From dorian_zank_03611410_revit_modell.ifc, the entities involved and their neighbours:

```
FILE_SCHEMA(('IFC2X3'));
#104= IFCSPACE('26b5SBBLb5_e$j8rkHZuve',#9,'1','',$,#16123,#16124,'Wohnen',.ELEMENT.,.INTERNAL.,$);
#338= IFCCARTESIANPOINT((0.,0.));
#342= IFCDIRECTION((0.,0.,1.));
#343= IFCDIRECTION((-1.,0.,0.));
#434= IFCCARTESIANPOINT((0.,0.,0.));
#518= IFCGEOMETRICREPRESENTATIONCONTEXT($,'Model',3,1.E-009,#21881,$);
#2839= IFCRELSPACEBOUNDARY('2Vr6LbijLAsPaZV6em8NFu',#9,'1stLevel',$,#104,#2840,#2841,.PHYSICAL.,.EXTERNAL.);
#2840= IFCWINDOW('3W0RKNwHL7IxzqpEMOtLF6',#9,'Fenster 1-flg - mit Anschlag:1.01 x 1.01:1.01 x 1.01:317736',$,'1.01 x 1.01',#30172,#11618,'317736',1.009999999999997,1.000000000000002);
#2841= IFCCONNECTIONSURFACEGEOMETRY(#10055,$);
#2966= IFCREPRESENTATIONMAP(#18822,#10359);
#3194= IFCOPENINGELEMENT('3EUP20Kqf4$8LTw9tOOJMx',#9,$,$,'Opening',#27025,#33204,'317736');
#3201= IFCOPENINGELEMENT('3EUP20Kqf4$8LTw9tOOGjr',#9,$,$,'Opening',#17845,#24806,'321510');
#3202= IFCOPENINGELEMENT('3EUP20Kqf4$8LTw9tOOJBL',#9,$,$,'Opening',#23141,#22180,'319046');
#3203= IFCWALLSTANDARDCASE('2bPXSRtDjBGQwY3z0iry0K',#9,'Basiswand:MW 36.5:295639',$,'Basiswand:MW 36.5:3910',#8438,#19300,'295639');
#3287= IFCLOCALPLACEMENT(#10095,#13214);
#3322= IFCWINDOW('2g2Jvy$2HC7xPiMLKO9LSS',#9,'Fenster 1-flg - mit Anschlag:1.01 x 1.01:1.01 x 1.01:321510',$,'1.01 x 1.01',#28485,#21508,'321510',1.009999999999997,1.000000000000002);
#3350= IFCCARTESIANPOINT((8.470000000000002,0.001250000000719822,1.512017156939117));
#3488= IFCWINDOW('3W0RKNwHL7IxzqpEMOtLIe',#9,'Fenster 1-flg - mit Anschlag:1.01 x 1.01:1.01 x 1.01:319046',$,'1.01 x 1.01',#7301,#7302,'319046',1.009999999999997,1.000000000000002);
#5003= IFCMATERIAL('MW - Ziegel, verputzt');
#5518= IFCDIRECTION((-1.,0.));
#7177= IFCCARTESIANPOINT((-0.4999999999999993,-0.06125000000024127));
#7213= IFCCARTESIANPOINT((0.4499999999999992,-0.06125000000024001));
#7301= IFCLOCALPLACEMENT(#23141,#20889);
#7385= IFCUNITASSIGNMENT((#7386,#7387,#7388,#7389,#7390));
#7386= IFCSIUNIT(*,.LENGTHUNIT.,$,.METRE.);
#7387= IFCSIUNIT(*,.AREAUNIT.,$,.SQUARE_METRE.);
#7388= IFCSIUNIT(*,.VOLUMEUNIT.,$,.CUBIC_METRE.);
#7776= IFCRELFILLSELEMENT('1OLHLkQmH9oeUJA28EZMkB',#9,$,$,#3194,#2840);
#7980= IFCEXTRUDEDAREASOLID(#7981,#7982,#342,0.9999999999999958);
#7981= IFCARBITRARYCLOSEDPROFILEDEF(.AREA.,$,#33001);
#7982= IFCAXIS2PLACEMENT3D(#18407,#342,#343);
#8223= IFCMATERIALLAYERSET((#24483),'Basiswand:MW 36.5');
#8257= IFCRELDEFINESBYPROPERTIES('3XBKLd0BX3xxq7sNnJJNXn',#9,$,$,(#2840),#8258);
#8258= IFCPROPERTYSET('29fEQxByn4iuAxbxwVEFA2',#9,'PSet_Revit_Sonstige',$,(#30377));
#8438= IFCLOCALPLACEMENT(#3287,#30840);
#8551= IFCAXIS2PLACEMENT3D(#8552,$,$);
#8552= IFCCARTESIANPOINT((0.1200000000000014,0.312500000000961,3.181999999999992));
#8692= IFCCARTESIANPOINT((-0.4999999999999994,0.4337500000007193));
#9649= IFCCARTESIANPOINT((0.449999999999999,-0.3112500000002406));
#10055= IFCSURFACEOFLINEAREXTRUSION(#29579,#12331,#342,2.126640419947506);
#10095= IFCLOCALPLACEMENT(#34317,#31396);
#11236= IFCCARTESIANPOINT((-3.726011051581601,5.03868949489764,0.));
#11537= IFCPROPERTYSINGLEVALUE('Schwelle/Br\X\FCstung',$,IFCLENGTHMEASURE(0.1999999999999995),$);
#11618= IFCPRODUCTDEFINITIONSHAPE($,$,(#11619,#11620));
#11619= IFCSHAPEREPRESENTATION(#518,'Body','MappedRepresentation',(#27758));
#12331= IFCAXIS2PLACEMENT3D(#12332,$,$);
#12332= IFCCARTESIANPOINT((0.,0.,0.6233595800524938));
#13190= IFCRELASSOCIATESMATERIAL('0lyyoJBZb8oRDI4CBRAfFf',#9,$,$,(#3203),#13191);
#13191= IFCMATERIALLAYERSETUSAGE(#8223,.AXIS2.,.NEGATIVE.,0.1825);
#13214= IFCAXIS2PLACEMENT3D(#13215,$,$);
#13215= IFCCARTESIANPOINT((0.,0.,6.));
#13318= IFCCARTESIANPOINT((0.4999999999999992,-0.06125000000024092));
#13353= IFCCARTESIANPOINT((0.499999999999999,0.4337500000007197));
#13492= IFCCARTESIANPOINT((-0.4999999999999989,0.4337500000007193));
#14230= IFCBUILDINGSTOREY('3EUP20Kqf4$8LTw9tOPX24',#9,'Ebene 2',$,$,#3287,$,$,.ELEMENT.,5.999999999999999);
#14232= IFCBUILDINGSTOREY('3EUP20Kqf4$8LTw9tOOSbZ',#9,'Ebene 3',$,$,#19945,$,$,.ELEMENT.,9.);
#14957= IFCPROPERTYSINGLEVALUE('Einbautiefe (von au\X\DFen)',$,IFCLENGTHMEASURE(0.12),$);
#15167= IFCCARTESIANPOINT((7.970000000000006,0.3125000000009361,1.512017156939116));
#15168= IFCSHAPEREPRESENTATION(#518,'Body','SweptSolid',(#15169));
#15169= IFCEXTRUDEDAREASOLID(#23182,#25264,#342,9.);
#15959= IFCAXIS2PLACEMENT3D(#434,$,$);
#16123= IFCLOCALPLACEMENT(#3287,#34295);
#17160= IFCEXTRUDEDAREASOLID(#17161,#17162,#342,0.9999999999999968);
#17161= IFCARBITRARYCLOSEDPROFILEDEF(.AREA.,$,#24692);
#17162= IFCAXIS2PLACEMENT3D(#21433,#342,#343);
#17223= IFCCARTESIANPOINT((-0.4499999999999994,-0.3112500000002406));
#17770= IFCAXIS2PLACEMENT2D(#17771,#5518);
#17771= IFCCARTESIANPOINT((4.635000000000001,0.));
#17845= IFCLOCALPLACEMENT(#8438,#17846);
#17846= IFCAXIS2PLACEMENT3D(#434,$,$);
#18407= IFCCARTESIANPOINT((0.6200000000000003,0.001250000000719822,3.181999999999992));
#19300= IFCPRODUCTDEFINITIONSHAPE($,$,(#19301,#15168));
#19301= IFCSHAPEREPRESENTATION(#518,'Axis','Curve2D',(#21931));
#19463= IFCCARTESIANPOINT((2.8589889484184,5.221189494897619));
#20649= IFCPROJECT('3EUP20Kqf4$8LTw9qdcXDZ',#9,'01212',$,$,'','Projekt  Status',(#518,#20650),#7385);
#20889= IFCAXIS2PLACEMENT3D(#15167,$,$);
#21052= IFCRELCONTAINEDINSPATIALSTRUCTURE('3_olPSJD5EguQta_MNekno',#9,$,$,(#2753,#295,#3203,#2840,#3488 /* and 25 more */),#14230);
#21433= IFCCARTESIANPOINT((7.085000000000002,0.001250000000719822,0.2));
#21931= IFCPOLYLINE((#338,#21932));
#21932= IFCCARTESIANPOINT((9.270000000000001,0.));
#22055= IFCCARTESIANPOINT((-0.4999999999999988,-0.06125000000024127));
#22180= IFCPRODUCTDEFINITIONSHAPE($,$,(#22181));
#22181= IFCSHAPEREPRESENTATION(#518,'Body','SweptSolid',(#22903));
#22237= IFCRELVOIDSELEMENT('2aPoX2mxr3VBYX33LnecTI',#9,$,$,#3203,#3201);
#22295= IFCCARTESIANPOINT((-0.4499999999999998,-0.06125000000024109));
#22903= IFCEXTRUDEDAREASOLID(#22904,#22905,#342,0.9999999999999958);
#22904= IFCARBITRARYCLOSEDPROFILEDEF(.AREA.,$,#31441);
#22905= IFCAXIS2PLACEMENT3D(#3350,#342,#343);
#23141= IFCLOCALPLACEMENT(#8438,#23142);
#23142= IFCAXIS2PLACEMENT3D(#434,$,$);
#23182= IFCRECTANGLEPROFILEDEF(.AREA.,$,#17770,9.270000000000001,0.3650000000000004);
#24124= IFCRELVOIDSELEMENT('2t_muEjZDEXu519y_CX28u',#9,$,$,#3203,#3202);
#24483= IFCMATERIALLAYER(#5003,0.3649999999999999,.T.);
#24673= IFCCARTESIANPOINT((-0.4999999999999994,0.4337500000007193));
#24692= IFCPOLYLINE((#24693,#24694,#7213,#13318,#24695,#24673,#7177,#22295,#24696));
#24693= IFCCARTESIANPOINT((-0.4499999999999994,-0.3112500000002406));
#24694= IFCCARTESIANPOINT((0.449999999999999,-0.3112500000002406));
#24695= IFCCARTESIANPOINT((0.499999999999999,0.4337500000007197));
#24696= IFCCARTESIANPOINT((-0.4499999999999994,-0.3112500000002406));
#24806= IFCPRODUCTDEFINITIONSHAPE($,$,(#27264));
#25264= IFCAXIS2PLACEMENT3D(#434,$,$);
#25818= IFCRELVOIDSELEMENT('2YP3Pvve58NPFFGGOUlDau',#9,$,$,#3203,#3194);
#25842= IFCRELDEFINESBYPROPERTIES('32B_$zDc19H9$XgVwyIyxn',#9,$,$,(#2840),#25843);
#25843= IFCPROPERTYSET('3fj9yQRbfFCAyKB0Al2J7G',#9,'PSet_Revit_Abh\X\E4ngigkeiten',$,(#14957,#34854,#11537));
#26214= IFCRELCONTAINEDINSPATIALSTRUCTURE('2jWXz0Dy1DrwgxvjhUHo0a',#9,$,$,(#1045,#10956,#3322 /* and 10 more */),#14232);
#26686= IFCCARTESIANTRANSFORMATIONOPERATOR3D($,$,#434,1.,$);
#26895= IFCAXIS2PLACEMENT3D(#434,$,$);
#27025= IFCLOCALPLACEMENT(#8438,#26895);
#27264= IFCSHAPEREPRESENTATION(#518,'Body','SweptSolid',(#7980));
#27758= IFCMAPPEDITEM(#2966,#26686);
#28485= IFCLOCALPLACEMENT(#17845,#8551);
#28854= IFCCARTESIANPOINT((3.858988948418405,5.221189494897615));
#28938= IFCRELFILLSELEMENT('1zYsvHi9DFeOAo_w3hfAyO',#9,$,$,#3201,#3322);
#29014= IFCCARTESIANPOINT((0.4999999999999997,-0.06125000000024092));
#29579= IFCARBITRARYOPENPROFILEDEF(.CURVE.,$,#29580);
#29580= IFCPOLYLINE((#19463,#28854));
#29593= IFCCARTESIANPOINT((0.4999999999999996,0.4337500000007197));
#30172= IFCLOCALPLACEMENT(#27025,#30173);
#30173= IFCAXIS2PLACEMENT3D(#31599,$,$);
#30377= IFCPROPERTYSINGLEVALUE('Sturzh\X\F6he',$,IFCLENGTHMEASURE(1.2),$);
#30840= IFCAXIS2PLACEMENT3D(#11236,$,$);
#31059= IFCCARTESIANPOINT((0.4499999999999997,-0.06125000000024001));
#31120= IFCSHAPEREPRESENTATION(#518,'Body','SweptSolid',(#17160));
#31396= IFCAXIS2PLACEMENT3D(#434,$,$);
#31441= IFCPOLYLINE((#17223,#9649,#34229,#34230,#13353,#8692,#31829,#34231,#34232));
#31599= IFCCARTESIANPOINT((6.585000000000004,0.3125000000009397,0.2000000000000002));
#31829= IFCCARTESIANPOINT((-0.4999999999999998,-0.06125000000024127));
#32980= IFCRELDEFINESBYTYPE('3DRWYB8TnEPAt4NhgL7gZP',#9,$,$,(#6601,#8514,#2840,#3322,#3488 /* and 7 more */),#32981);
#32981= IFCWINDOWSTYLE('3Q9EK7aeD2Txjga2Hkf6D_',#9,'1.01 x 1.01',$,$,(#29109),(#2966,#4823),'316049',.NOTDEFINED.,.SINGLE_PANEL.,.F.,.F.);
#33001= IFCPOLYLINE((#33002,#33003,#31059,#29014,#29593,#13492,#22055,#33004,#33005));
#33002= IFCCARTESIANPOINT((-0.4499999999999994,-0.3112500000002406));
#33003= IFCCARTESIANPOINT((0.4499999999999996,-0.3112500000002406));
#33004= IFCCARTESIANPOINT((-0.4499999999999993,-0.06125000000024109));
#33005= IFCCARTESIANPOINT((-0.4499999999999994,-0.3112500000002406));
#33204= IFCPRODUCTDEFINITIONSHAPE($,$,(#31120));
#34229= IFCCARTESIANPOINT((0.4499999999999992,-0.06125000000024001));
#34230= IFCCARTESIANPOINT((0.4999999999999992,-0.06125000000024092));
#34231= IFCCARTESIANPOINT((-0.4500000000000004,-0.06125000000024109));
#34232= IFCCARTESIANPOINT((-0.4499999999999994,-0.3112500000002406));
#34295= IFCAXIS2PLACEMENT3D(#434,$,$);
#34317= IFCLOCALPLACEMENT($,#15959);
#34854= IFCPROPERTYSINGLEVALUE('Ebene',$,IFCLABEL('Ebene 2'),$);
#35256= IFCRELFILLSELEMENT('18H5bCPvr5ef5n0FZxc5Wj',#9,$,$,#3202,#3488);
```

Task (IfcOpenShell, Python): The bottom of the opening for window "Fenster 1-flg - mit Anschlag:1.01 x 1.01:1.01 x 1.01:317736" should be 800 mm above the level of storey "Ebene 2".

```python
import numpy as np
import ifcopenshell
import ifcopenshell.api.geometry
import ifcopenshell.api.pset
import ifcopenshell.geom
import ifcopenshell.util.element
import ifcopenshell.util.placement
import ifcopenshell.util.shape
import ifcopenshell.util.unit

model = ifcopenshell.open("dorian_zank_03611410_revit_modell.ifc")
unit_scale = ifcopenshell.util.unit.calculate_unit_scale(model)

window = model.by_id(2840)
opening = window.FillsVoids[0].RelatingOpeningElement
storey = ifcopenshell.util.element.get_container(window, ifc_class="IfcBuildingStorey")
level = ifcopenshell.util.placement.get_local_placement(storey.ObjectPlacement)[2, 3]

# The opening's origin need not be at the sill, so measure its lowest point.
shape = ifcopenshell.geom.create_shape(ifcopenshell.geom.settings(), opening)
bottom = ifcopenshell.util.shape.get_shape_bottom_elevation(shape, shape.geometry) / unit_scale
dz = level + 0.8 / unit_scale - bottom

shift = np.array([0.0, 0.0, dz])
# The window is placed relative to its opening, so it follows when the opening moves.
matrix = ifcopenshell.util.placement.get_local_placement(opening.ObjectPlacement)
matrix[:3, 3] += shift
ifcopenshell.api.geometry.edit_object_placement(
    model, product=opening, matrix=matrix, is_si=False, should_transform_children=True
)

# Space boundary surfaces are stored in each space's coordinates; move them too.
for rel in window.ProvidesBoundaries:
    if not rel.ConnectionGeometry:
        continue
    surface = rel.ConnectionGeometry.SurfaceOnRelatingElement
    space_matrix = ifcopenshell.util.placement.get_local_placement(rel.RelatingSpace.ObjectPlacement)
    point = np.array(surface.Position.Location.Coordinates) + space_matrix[:3, :3].T @ shift
    surface.Position = model.createIfcAxis2Placement3D(
        model.createIfcCartesianPoint(point.tolist()), surface.Position.Axis, surface.Position.RefDirection
    )

# Keep the stored heights in step.
pset = model.by_id(ifcopenshell.util.element.get_pset(window, "PSet_Revit_Sonstige", should_inherit=False)["id"])
ifcopenshell.api.pset.edit_pset(model, pset=pset, properties={
    "Sturzhöhe": model.create_entity("IfcLengthMeasure", ifcopenshell.util.element.get_pset(window, "PSet_Revit_Sonstige", "Sturzhöhe") + dz),
})
pset = model.by_id(ifcopenshell.util.element.get_pset(window, "PSet_Revit_Abhängigkeiten", should_inherit=False)["id"])
ifcopenshell.api.pset.edit_pset(model, pset=pset, properties={
    "Schwelle/Brüstung": model.create_entity("IfcLengthMeasure", ifcopenshell.util.element.get_pset(window, "PSet_Revit_Abhängigkeiten", "Schwelle/Brüstung") + dz),
})

print(f"moved by {dz * unit_scale:+.3f} m")

model.write("dorian_zank_03611410_revit_modell_edited.ifc")
```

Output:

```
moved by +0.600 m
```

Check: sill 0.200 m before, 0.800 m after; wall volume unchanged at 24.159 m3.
